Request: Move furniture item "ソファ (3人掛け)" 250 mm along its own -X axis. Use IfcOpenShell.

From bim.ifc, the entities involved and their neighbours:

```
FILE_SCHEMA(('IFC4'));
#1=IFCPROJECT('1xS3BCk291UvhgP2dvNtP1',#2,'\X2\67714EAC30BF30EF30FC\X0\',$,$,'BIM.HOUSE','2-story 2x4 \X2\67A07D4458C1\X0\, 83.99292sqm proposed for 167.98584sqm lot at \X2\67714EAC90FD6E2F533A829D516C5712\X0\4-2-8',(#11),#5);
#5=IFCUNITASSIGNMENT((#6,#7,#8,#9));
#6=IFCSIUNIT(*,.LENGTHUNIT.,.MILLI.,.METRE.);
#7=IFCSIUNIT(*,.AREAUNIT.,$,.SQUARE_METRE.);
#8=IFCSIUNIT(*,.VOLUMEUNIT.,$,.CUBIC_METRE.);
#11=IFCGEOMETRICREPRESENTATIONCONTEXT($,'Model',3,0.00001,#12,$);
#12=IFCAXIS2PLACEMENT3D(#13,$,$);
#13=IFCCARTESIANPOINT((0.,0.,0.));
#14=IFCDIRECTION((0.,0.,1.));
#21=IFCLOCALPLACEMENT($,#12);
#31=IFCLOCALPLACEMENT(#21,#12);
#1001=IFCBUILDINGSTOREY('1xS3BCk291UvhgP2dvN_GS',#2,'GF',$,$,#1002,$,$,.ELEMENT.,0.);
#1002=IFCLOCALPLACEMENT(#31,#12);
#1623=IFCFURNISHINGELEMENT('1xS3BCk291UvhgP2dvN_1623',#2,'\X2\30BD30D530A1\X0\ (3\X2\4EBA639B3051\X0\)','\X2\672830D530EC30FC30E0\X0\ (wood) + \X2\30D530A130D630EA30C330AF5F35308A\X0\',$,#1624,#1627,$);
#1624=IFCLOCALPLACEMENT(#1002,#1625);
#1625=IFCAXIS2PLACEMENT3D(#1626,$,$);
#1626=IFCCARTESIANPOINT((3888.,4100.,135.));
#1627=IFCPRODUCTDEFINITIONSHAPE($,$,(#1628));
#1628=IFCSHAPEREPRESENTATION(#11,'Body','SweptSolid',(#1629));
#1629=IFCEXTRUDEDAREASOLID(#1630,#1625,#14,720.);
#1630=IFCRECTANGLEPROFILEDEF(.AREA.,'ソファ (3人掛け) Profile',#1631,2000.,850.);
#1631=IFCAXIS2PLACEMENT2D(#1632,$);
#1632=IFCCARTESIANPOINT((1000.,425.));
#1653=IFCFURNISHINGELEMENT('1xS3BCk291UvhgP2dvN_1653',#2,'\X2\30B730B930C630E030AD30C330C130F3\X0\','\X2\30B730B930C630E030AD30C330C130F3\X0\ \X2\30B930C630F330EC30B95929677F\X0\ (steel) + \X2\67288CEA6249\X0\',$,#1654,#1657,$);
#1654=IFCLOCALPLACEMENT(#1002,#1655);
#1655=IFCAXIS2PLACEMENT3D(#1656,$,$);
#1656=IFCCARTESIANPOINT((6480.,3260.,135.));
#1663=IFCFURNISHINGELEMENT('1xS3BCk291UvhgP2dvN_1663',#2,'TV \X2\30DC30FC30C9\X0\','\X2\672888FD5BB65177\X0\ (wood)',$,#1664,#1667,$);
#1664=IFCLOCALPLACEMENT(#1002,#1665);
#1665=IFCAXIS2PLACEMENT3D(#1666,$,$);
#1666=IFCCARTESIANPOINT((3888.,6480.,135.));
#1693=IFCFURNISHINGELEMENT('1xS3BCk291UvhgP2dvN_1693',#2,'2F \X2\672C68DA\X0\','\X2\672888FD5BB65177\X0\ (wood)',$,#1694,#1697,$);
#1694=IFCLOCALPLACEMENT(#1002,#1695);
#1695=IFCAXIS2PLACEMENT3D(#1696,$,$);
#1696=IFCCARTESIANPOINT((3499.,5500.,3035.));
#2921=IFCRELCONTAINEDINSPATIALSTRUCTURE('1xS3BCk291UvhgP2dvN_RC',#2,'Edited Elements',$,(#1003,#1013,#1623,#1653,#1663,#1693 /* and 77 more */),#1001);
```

```python
import ifcopenshell
import ifcopenshell.api.geometry
import ifcopenshell.util.placement
import ifcopenshell.util.unit

model = ifcopenshell.open("bim.ifc")
unit_scale = ifcopenshell.util.unit.calculate_unit_scale(model)

item = model.by_id(1623)
matrix = ifcopenshell.util.placement.get_local_placement(item.ObjectPlacement)
matrix[:3, 3] -= matrix[:3, 0] * 0.25 / unit_scale
ifcopenshell.api.geometry.edit_object_placement(model, product=item, matrix=matrix, is_si=False)

print(ifcopenshell.util.placement.get_local_placement(item.ObjectPlacement).round(3) + 0.0)

model.write("bim_updated.ifc")
```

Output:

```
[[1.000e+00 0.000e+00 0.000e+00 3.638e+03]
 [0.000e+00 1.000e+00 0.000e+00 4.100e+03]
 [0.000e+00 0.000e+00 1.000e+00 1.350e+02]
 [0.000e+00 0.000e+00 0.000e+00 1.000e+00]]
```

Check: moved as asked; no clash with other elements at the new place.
